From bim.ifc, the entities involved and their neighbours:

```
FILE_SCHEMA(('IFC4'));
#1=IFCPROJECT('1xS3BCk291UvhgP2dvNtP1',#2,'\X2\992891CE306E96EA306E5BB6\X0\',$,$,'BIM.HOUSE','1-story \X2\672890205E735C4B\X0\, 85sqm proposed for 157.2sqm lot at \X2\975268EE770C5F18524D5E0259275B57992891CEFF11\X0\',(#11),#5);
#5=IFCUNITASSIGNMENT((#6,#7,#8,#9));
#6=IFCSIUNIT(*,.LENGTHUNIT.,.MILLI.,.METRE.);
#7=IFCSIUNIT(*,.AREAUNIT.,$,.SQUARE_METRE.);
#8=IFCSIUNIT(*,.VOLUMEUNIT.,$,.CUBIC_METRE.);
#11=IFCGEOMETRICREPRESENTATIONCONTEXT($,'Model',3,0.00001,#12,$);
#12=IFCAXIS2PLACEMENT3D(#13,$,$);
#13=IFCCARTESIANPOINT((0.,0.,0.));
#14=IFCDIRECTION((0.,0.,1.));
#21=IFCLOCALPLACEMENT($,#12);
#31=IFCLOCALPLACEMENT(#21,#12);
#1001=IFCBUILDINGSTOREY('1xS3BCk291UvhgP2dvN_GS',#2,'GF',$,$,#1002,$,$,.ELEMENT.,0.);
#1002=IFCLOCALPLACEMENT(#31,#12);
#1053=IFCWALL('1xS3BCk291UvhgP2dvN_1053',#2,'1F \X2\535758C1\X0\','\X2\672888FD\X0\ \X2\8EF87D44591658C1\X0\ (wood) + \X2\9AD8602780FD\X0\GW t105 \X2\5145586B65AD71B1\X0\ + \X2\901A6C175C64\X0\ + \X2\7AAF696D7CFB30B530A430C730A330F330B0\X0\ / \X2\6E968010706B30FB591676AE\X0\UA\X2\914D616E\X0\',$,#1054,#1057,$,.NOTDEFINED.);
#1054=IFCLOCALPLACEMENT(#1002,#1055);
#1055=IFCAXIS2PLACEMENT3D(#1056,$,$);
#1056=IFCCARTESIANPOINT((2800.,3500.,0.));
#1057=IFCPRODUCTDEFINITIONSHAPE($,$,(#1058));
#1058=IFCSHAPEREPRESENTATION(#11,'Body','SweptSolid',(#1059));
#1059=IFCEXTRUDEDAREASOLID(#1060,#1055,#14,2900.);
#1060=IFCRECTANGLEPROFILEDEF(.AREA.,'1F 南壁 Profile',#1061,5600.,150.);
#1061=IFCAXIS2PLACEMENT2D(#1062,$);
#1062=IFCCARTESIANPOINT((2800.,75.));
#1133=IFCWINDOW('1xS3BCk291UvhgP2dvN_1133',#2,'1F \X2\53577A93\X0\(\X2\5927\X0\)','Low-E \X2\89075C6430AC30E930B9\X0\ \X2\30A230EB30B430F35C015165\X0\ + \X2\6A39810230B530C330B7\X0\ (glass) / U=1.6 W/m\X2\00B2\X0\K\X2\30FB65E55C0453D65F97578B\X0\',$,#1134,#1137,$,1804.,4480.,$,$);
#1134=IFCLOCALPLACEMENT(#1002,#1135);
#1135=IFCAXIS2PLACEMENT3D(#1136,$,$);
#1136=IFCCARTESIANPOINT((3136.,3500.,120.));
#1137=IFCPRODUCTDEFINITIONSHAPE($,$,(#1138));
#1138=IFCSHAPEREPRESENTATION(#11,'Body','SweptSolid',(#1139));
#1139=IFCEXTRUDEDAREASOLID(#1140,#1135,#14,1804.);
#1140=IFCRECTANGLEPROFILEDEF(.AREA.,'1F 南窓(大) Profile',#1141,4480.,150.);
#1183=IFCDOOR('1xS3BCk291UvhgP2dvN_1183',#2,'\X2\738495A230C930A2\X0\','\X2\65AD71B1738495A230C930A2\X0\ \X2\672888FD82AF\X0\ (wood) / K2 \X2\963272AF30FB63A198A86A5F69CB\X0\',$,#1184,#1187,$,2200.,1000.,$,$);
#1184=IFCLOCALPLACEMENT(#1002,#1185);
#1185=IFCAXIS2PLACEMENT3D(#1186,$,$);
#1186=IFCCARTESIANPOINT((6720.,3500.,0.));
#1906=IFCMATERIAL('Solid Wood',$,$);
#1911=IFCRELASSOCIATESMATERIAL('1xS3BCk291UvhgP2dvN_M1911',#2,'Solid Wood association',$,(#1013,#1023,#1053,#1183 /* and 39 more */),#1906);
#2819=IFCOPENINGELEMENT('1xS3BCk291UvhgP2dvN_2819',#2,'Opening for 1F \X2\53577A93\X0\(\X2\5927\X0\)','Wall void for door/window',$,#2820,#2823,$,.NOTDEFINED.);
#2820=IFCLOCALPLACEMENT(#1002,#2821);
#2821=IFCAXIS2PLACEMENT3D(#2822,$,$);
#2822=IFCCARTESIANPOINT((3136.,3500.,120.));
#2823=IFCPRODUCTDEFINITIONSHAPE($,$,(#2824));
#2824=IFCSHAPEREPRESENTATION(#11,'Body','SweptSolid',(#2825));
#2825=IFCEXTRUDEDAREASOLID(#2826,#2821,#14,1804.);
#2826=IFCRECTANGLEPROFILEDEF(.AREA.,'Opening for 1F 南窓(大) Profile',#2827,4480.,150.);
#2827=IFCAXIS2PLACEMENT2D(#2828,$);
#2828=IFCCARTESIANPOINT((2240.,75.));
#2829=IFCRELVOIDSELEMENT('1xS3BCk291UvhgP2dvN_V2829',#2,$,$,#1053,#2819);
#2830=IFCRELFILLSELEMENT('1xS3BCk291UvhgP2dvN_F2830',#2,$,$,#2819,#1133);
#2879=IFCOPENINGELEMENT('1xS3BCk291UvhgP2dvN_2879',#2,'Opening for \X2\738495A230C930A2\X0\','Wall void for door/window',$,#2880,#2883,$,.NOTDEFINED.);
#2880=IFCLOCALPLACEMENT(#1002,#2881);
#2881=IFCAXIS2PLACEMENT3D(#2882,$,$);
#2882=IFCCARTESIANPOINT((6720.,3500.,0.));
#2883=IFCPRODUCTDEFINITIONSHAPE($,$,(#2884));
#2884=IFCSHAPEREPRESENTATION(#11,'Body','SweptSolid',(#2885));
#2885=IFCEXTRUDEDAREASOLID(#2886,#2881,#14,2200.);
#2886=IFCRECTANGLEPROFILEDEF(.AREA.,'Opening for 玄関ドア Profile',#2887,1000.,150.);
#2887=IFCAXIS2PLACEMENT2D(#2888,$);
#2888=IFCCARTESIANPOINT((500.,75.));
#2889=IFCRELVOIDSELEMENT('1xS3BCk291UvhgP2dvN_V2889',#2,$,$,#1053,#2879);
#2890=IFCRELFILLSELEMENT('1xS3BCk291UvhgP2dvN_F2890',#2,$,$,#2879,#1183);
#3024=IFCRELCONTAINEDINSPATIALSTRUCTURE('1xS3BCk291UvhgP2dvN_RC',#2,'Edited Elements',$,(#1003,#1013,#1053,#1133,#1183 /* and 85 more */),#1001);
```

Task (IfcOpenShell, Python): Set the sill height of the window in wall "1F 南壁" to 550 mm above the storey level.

```python
import numpy as np
import ifcopenshell
import ifcopenshell.api.geometry
import ifcopenshell.geom
import ifcopenshell.util.element
import ifcopenshell.util.placement
import ifcopenshell.util.shape
import ifcopenshell.util.unit

model = ifcopenshell.open("bim.ifc")
unit_scale = ifcopenshell.util.unit.calculate_unit_scale(model)

window = model.by_guid("1xS3BCk291UvhgP2dvN_1133")
opening = window.FillsVoids[0].RelatingOpeningElement
storey = ifcopenshell.util.element.get_container(window, ifc_class="IfcBuildingStorey")
level = ifcopenshell.util.placement.get_local_placement(storey.ObjectPlacement)[2, 3]

# The opening's origin need not be at the sill, so measure its lowest point.
shape = ifcopenshell.geom.create_shape(ifcopenshell.geom.settings(), opening)
bottom = ifcopenshell.util.shape.get_shape_bottom_elevation(shape, shape.geometry) / unit_scale
dz = level + 550.0 - bottom

shift = np.array([0.0, 0.0, dz])
# The window is not placed relative to its opening, so move both.
for product in (opening, window):
    matrix = ifcopenshell.util.placement.get_local_placement(product.ObjectPlacement)
    matrix[:3, 3] += shift
    ifcopenshell.api.geometry.edit_object_placement(model, product=product, matrix=matrix, is_si=False)

print(f"moved by {dz * unit_scale:+.3f} m")

model.write("bim_edited.ifc")
```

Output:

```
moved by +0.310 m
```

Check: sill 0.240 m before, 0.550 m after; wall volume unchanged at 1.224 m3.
